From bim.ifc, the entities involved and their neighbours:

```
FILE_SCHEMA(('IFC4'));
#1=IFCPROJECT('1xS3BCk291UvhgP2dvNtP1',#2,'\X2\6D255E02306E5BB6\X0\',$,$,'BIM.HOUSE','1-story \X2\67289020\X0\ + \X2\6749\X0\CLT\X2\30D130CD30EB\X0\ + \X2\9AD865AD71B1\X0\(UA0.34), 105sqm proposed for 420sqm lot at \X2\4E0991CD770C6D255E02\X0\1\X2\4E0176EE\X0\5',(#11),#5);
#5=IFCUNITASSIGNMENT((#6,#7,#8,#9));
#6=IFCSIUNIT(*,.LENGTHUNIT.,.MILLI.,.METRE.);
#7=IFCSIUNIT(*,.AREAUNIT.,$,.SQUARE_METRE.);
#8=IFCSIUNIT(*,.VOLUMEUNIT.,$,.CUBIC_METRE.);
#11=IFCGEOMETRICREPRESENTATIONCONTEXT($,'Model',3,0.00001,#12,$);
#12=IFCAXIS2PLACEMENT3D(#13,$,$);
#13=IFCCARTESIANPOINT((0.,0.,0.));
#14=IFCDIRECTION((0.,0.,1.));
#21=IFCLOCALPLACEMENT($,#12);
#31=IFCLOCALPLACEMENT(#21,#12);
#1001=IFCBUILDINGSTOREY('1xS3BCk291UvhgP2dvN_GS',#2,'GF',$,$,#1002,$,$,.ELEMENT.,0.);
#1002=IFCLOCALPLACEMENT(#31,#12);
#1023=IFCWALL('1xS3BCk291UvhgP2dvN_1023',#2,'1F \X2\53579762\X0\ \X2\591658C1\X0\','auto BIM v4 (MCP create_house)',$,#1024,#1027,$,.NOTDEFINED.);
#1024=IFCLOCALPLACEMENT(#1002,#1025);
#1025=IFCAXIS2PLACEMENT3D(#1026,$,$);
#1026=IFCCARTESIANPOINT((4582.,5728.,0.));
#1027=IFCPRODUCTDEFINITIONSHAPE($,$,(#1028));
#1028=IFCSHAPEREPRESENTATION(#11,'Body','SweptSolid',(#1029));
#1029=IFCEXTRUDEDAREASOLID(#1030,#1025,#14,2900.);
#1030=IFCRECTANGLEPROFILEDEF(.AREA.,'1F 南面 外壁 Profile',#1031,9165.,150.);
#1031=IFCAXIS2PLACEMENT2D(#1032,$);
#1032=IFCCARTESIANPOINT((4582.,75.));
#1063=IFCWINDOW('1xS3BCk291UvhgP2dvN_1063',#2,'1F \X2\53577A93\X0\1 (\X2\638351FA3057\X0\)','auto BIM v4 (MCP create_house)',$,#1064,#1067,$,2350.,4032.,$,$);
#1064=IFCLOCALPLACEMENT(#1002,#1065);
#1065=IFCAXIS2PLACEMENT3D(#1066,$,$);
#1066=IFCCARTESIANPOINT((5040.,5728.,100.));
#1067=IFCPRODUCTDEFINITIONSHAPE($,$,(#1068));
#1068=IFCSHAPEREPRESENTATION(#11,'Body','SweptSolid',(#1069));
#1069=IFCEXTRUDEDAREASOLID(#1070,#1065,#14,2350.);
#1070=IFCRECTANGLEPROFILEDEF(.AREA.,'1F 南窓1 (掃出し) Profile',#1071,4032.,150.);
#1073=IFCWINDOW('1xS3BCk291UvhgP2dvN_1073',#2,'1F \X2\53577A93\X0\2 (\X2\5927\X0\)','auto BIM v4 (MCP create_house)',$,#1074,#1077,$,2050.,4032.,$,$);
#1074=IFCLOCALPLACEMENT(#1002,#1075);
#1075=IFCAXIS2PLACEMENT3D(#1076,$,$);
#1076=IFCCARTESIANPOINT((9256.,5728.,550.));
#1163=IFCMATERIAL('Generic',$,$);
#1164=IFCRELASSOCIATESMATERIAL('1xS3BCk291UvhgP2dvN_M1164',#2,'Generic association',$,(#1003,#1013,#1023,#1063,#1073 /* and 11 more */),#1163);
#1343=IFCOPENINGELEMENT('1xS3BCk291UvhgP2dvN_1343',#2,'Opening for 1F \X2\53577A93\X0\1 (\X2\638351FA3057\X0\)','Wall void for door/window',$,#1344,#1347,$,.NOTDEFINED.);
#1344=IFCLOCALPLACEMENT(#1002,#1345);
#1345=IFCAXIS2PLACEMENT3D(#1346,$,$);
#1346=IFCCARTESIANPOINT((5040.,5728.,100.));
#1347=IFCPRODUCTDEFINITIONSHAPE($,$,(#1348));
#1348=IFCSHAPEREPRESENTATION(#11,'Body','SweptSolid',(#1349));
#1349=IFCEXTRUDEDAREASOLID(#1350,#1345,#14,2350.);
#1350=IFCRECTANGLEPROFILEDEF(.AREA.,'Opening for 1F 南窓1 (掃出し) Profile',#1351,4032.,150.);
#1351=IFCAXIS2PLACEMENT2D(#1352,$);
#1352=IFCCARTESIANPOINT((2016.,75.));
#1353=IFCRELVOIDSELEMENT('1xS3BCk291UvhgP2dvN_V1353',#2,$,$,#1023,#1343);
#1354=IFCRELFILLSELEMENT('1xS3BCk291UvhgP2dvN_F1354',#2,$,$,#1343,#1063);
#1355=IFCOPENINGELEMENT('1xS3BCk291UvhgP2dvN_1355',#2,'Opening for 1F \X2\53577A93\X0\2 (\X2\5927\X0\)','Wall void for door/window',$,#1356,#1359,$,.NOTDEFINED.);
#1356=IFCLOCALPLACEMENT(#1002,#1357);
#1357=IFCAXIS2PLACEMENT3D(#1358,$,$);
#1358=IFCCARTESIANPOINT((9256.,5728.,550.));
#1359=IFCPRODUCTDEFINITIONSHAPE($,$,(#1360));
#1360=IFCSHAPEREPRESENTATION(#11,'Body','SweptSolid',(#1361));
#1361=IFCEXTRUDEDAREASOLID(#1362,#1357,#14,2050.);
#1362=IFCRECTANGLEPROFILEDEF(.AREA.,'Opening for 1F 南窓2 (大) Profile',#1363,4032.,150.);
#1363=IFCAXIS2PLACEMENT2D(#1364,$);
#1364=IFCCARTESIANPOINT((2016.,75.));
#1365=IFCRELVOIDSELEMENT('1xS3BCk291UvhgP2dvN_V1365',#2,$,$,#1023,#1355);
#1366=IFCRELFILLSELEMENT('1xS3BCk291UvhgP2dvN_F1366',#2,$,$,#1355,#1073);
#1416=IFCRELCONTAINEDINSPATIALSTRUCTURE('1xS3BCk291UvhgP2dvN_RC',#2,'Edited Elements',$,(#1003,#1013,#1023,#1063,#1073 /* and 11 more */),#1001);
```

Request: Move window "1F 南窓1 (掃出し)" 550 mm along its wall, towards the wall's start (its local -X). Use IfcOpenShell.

```python
import ifcopenshell
import ifcopenshell.api.geometry
import ifcopenshell.util.placement

model = ifcopenshell.open("bim.ifc")

window = model.by_guid("1xS3BCk291UvhgP2dvN_1063")
opening = window.FillsVoids[0].RelatingOpeningElement
wall = opening.VoidsElements[0].RelatingBuildingElement

wall_matrix = ifcopenshell.util.placement.get_local_placement(wall.ObjectPlacement)
shift = wall_matrix[:3, 0] * -550.0
before = ifcopenshell.util.placement.get_local_placement(window.ObjectPlacement)[:3, 3].copy()

# The window is not placed relative to its opening, so move both.
for product in (opening, window):
    matrix = ifcopenshell.util.placement.get_local_placement(product.ObjectPlacement)
    matrix[:3, 3] += shift
    ifcopenshell.api.geometry.edit_object_placement(model, product=product, matrix=matrix, is_si=False)

after = ifcopenshell.util.placement.get_local_placement(window.ObjectPlacement)[:3, 3]
print("window moved by", (after - before).round(3) + 0.0)

model.write("bim_rev.ifc")
```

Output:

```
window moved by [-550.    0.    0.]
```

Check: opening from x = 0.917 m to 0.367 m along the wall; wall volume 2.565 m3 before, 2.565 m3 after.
